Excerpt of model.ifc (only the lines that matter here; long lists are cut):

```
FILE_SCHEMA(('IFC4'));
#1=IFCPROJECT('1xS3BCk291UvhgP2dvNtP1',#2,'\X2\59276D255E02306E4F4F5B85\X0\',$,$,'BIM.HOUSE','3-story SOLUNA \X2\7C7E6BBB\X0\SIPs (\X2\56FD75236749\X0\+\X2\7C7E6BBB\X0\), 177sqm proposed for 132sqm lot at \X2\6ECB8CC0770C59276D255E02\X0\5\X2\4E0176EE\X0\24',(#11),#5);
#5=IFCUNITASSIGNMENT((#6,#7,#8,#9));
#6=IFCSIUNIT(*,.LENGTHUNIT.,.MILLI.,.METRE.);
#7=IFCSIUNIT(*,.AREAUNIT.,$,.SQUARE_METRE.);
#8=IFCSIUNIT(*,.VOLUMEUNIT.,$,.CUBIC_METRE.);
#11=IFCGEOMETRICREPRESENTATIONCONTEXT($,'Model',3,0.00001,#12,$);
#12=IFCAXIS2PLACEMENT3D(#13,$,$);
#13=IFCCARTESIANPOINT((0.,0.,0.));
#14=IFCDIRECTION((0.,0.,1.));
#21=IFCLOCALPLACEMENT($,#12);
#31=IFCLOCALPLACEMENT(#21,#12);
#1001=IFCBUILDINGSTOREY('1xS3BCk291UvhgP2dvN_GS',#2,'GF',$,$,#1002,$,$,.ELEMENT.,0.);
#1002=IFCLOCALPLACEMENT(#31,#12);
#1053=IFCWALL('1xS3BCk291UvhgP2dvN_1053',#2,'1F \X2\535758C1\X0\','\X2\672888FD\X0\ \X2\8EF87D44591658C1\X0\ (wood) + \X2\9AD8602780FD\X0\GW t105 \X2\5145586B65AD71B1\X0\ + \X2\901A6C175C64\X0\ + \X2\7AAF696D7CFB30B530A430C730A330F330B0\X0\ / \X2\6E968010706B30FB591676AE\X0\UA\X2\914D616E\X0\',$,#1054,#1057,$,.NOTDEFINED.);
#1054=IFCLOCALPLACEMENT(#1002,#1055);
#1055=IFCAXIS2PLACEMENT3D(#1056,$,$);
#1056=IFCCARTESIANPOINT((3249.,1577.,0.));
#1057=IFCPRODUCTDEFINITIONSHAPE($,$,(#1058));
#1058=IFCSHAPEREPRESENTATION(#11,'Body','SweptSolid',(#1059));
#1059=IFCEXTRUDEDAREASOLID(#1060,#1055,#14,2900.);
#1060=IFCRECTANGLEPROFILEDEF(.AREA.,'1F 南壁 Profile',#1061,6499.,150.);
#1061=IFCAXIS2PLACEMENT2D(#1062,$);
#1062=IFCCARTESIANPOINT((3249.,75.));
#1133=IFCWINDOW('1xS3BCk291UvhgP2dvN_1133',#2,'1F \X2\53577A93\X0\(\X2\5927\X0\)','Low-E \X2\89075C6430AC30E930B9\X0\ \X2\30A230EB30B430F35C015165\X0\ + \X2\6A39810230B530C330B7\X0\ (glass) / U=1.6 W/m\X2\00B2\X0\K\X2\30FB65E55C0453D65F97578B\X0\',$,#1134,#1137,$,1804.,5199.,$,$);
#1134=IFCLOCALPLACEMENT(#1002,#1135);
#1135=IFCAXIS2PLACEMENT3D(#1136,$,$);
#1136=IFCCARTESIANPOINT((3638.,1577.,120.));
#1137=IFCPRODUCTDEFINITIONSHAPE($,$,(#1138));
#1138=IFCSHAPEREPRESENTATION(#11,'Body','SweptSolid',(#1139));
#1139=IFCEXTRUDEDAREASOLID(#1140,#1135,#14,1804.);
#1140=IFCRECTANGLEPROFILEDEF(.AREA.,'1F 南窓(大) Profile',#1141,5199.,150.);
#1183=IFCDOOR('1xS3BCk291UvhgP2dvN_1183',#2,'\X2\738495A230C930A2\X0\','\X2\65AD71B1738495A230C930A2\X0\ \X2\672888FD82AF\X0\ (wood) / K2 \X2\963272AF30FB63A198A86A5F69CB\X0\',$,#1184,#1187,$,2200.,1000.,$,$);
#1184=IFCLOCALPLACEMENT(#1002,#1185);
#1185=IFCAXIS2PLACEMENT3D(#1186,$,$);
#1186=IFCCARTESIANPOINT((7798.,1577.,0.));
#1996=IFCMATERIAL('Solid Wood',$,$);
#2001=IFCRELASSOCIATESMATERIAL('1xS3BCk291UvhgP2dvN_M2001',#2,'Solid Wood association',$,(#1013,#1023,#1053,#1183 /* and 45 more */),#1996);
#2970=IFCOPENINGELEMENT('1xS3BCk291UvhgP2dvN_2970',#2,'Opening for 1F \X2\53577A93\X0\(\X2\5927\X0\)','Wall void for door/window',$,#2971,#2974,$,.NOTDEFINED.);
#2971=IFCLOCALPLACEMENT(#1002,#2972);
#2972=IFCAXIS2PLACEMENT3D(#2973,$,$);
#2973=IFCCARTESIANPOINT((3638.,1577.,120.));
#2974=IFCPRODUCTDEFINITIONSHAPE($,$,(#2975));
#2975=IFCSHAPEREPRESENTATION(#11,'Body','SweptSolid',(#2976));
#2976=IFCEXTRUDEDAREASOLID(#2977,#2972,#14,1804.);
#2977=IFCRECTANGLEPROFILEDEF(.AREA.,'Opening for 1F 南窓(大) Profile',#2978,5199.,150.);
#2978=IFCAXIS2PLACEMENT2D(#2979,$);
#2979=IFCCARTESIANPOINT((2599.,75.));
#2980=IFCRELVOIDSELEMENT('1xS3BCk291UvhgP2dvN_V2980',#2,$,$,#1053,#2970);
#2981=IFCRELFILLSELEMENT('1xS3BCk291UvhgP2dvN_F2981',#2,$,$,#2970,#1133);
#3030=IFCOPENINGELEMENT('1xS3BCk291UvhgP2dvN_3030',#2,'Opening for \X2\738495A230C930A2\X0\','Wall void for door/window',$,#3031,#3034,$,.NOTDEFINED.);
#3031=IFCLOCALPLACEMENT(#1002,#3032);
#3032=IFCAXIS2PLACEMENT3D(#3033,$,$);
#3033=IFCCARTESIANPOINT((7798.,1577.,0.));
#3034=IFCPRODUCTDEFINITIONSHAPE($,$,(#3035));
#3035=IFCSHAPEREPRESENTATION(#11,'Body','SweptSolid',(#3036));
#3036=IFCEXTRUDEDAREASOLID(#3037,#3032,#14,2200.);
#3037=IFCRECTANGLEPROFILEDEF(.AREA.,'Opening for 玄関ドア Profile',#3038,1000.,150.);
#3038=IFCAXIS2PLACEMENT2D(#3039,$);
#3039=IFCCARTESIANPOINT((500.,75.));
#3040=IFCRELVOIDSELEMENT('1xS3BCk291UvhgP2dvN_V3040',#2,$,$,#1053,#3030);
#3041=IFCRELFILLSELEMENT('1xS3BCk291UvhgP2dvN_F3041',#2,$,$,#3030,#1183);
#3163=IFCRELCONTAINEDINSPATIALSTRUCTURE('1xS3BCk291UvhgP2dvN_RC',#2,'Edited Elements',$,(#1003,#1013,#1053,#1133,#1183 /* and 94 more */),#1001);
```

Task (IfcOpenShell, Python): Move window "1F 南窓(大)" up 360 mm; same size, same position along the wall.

```python
import numpy as np
import ifcopenshell
import ifcopenshell.api.geometry
import ifcopenshell.util.placement
import ifcopenshell.util.unit

model = ifcopenshell.open("model.ifc")
unit_scale = ifcopenshell.util.unit.calculate_unit_scale(model)

window = model.by_guid("1xS3BCk291UvhgP2dvN_1133")
opening = window.FillsVoids[0].RelatingOpeningElement
dz = 0.36 / unit_scale

shift = np.array([0.0, 0.0, dz])
# The window is not placed relative to its opening, so move both.
for product in (opening, window):
    matrix = ifcopenshell.util.placement.get_local_placement(product.ObjectPlacement)
    matrix[:3, 3] += shift
    ifcopenshell.api.geometry.edit_object_placement(model, product=product, matrix=matrix, is_si=False)

print(f"moved by {dz * unit_scale:+.3f} m")

model.write("model-out.ifc")
```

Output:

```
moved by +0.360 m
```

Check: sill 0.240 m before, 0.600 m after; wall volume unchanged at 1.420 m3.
